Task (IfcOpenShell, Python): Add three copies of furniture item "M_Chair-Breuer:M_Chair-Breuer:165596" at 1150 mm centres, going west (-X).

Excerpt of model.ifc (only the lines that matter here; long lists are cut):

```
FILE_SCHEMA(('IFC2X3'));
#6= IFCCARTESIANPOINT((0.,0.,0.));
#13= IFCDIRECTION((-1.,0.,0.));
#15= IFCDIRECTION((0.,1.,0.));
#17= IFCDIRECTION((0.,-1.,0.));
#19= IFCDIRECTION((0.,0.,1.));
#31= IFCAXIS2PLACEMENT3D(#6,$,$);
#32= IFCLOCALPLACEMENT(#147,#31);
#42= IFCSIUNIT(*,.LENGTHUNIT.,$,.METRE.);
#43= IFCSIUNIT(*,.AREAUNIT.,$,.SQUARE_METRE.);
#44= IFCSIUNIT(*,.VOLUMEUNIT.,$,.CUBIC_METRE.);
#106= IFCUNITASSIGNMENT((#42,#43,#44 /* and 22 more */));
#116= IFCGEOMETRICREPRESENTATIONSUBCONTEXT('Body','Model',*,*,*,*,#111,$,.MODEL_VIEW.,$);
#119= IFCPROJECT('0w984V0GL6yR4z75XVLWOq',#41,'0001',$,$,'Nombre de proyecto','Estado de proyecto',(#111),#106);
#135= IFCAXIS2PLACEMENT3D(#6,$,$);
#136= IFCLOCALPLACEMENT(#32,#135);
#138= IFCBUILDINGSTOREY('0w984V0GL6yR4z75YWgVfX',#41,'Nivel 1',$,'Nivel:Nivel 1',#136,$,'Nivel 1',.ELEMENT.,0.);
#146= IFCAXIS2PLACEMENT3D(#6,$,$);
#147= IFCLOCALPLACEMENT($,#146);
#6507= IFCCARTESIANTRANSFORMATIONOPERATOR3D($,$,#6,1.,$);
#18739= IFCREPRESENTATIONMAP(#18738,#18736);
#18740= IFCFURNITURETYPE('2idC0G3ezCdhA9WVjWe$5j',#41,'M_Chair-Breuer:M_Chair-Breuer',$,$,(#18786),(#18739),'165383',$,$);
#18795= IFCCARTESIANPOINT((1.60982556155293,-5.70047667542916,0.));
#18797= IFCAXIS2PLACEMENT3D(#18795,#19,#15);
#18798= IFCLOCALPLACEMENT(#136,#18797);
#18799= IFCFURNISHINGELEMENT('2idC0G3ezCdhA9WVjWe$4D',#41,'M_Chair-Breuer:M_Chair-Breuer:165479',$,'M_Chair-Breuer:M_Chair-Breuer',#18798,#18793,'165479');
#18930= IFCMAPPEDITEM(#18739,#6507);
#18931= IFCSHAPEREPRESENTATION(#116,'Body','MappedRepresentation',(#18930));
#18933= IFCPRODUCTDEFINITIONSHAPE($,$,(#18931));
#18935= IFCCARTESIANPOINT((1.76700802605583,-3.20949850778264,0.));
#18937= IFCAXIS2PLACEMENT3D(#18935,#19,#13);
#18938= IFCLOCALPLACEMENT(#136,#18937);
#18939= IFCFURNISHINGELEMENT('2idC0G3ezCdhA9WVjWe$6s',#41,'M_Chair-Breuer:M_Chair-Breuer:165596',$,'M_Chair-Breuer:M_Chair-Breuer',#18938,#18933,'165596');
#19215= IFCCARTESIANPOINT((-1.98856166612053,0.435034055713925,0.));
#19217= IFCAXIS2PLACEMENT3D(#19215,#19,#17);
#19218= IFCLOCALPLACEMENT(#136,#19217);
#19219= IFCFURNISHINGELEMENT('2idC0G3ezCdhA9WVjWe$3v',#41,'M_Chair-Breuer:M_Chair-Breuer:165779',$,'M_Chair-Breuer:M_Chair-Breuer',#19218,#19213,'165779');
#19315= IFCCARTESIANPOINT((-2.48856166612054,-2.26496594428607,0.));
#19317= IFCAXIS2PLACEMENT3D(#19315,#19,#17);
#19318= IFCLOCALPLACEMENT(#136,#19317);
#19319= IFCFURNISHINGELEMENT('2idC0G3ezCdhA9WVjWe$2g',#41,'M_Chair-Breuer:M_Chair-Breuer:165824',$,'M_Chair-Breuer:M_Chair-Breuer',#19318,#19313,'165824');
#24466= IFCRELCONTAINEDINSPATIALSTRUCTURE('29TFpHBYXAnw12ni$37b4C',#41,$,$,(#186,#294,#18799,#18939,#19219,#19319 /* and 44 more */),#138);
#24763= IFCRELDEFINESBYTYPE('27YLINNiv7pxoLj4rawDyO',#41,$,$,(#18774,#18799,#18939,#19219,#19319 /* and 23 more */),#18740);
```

```python
import numpy as np
import ifcopenshell
import ifcopenshell.api.geometry
import ifcopenshell.api.root
import ifcopenshell.util.element
import ifcopenshell.util.placement
import ifcopenshell.util.unit

model = ifcopenshell.open("model.ifc")
unit_scale = ifcopenshell.util.unit.calculate_unit_scale(model)


def reuse_history(source, copy):
    """copy_class also copies each property set's owner history, people and application; keep the originals."""
    for rel in copy.IsDefinedBy:
        if rel.is_a("IfcRelDefinesByProperties") and (history := rel.RelatingPropertyDefinition.OwnerHistory):
            rel.RelatingPropertyDefinition.OwnerHistory = source.OwnerHistory
            ifcopenshell.util.element.remove_deep2(model, history)


source = model.by_guid("2idC0G3ezCdhA9WVjWe$6s")
base = ifcopenshell.util.placement.get_local_placement(source.ObjectPlacement)
step = np.array([-1.0, 0.0, 0.0]) * 1.15 / unit_scale

for i in range(1, 4):
    copy = ifcopenshell.api.root.copy_class(model, product=source)
    copy.Representation = ifcopenshell.util.element.copy_deep(
        model, source.Representation, exclude=["IfcGeometricRepresentationContext", "IfcRepresentationMap"]
    )
    copy.Name = "M_Chair-Breuer:M_Chair-Breuer"
    copy.Tag = None
    reuse_history(source, copy)
    matrix = base.copy()
    matrix[:3, 3] += i * step
    print("added at", matrix[:3, 3].round(3) + 0.0)
    ifcopenshell.api.geometry.edit_object_placement(model, product=copy, matrix=matrix, is_si=False)

model.write("model_edited.ifc")
```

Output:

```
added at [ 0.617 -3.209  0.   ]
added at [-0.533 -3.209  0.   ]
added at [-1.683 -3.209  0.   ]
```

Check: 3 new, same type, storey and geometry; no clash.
